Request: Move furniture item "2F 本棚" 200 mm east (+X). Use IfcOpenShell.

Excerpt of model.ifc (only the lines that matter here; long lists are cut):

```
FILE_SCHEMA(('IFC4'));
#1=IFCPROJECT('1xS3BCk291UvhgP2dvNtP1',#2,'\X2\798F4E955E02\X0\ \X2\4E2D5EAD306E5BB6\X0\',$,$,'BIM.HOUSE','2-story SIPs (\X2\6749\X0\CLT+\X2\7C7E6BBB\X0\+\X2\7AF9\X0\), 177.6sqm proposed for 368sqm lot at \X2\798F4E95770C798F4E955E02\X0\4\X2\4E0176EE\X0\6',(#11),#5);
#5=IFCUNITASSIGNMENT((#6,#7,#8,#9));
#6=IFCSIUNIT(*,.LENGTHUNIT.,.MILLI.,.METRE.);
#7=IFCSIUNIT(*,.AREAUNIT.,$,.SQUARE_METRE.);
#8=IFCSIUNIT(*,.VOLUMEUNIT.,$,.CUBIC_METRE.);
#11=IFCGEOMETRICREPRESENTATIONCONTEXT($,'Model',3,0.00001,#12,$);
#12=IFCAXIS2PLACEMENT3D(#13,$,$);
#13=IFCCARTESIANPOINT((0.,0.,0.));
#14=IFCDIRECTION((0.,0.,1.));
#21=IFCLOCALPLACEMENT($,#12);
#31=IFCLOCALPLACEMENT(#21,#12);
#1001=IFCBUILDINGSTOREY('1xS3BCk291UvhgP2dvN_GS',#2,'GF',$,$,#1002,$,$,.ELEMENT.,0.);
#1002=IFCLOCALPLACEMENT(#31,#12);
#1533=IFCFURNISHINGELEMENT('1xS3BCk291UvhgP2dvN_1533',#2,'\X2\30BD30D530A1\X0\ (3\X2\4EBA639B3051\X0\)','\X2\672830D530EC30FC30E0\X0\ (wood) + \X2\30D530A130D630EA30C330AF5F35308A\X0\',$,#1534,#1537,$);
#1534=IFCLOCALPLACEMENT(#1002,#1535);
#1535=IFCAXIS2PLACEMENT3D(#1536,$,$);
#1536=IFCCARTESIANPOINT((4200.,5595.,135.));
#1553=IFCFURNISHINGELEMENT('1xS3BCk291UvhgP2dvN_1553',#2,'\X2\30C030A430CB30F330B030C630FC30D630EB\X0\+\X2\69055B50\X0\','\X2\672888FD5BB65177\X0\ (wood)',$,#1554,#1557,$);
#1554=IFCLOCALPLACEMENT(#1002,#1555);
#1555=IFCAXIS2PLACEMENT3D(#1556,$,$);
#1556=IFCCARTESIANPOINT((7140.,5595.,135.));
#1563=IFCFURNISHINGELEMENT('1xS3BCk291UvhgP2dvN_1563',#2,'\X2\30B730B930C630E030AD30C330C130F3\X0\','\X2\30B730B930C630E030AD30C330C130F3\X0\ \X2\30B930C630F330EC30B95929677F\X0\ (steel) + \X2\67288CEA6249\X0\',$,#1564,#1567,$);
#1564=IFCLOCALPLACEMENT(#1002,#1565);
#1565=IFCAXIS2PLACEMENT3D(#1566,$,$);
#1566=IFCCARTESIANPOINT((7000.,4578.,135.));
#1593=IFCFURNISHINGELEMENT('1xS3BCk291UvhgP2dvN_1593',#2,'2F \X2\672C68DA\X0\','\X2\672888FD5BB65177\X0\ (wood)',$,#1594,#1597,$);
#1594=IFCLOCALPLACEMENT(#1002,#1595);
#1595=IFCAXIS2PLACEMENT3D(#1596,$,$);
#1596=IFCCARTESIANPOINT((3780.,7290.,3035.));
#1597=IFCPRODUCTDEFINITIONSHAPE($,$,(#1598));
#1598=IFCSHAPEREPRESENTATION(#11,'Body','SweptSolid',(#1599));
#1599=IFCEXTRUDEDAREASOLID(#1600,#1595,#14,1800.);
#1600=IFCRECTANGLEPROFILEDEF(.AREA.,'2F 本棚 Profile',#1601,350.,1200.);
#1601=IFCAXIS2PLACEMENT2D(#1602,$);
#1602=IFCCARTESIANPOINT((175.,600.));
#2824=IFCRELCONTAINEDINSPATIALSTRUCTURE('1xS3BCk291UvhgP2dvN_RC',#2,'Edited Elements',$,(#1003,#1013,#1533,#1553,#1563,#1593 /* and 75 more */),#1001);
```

```python
import ifcopenshell
import ifcopenshell.api.geometry
import ifcopenshell.util.placement
import ifcopenshell.util.unit

model = ifcopenshell.open("model.ifc")
unit_scale = ifcopenshell.util.unit.calculate_unit_scale(model)

item = model.by_id(1593)
matrix = ifcopenshell.util.placement.get_local_placement(item.ObjectPlacement)
matrix[0, 3] += 0.2 / unit_scale
ifcopenshell.api.geometry.edit_object_placement(model, product=item, matrix=matrix, is_si=False)

print(ifcopenshell.util.placement.get_local_placement(item.ObjectPlacement).round(3) + 0.0)

model.write("model_rev.ifc")
```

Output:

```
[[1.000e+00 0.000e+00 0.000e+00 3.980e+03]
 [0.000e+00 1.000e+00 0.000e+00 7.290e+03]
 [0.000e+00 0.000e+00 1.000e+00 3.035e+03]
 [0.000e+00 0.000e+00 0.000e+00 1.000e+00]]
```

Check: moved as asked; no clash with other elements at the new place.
